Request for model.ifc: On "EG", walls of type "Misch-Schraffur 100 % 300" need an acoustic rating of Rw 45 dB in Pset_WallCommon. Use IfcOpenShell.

First a look at what the model holds.

```python
import ifcopenshell
import ifcopenshell.util.element

model = ifcopenshell.open("model.ifc")
print(model.schema)
storey = next(s for s in model.by_type("IfcBuildingStorey") if s.Name == "EG")
walls = [e for e in ifcopenshell.util.element.get_decomposition(storey) if e.is_a("IfcWall")]
seen = {}
for e in walls:
    element_type = ifcopenshell.util.element.get_type(e)
    key = (element_type.Name if element_type != e and element_type else None, ifcopenshell.util.element.get_pset(e, "Pset_WallCommon", "AcousticRating"))
    seen[key] = seen.get(key, 0) + 1
for (name, value), count in sorted(seen.items(), key=str):
    print(count, "x", name, "|", value)
```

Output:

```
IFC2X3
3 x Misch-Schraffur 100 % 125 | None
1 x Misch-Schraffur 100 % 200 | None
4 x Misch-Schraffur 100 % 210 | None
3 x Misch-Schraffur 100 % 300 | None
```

```python
import ifcopenshell
import ifcopenshell.api.pset
import ifcopenshell.util.element

model = ifcopenshell.open("model.ifc")

storey = next(s for s in model.by_type("IfcBuildingStorey") if s.Name == "EG")
walls = [e for e in ifcopenshell.util.element.get_decomposition(storey) if e.is_a("IfcWall")]

count = 0
for e in walls:
    element_type = ifcopenshell.util.element.get_type(e)
    if element_type in (None, e) or element_type.Name != "Misch-Schraffur 100 % 300":
        continue
    # add_pset returns the element's existing set when there is one.
    pset = ifcopenshell.api.pset.add_pset(model, product=e, name="Pset_WallCommon")
    ifcopenshell.api.pset.edit_pset(model, pset=pset, properties={"AcousticRating": "Rw 45 dB"})
    count += 1

print(count, "walls updated")

model.write("model_edited.ifc")
```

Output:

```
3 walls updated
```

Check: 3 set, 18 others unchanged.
